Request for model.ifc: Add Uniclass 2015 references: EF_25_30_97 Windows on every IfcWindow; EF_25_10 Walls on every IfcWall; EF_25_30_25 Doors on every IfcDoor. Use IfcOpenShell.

First a look at what the model holds.

```python
import ifcopenshell

model = ifcopenshell.open("model.ifc")
print(model.schema)
print("classifications:", [c.Name for c in model.by_type("IfcClassification")])
for ifc_class in ("IfcDoor", "IfcRoof", "IfcStair", "IfcWall", "IfcWindow"):
    print(ifc_class, len(model.by_type(ifc_class)))
```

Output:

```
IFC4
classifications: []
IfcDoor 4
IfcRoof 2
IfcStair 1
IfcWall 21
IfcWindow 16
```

```python
import ifcopenshell
import ifcopenshell.api.classification

model = ifcopenshell.open("model.ifc")

system = ifcopenshell.api.classification.add_classification(model, classification="Uniclass 2015")

codes = {
    "IfcWindow": ("EF_25_30_97", "Windows"),
    "IfcWall": ("EF_25_10", "Walls"),
    "IfcDoor": ("EF_25_30_25", "Doors"),
}
for ifc_class, (code, name) in codes.items():
    products = model.by_type(ifc_class)
    ifcopenshell.api.classification.add_reference(
        model, products=products, classification=system, identification=code, name=name
    )
    print(code, len(products))

model.write("model_rev.ifc")
```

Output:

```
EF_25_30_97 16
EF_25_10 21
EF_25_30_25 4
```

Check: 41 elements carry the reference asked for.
